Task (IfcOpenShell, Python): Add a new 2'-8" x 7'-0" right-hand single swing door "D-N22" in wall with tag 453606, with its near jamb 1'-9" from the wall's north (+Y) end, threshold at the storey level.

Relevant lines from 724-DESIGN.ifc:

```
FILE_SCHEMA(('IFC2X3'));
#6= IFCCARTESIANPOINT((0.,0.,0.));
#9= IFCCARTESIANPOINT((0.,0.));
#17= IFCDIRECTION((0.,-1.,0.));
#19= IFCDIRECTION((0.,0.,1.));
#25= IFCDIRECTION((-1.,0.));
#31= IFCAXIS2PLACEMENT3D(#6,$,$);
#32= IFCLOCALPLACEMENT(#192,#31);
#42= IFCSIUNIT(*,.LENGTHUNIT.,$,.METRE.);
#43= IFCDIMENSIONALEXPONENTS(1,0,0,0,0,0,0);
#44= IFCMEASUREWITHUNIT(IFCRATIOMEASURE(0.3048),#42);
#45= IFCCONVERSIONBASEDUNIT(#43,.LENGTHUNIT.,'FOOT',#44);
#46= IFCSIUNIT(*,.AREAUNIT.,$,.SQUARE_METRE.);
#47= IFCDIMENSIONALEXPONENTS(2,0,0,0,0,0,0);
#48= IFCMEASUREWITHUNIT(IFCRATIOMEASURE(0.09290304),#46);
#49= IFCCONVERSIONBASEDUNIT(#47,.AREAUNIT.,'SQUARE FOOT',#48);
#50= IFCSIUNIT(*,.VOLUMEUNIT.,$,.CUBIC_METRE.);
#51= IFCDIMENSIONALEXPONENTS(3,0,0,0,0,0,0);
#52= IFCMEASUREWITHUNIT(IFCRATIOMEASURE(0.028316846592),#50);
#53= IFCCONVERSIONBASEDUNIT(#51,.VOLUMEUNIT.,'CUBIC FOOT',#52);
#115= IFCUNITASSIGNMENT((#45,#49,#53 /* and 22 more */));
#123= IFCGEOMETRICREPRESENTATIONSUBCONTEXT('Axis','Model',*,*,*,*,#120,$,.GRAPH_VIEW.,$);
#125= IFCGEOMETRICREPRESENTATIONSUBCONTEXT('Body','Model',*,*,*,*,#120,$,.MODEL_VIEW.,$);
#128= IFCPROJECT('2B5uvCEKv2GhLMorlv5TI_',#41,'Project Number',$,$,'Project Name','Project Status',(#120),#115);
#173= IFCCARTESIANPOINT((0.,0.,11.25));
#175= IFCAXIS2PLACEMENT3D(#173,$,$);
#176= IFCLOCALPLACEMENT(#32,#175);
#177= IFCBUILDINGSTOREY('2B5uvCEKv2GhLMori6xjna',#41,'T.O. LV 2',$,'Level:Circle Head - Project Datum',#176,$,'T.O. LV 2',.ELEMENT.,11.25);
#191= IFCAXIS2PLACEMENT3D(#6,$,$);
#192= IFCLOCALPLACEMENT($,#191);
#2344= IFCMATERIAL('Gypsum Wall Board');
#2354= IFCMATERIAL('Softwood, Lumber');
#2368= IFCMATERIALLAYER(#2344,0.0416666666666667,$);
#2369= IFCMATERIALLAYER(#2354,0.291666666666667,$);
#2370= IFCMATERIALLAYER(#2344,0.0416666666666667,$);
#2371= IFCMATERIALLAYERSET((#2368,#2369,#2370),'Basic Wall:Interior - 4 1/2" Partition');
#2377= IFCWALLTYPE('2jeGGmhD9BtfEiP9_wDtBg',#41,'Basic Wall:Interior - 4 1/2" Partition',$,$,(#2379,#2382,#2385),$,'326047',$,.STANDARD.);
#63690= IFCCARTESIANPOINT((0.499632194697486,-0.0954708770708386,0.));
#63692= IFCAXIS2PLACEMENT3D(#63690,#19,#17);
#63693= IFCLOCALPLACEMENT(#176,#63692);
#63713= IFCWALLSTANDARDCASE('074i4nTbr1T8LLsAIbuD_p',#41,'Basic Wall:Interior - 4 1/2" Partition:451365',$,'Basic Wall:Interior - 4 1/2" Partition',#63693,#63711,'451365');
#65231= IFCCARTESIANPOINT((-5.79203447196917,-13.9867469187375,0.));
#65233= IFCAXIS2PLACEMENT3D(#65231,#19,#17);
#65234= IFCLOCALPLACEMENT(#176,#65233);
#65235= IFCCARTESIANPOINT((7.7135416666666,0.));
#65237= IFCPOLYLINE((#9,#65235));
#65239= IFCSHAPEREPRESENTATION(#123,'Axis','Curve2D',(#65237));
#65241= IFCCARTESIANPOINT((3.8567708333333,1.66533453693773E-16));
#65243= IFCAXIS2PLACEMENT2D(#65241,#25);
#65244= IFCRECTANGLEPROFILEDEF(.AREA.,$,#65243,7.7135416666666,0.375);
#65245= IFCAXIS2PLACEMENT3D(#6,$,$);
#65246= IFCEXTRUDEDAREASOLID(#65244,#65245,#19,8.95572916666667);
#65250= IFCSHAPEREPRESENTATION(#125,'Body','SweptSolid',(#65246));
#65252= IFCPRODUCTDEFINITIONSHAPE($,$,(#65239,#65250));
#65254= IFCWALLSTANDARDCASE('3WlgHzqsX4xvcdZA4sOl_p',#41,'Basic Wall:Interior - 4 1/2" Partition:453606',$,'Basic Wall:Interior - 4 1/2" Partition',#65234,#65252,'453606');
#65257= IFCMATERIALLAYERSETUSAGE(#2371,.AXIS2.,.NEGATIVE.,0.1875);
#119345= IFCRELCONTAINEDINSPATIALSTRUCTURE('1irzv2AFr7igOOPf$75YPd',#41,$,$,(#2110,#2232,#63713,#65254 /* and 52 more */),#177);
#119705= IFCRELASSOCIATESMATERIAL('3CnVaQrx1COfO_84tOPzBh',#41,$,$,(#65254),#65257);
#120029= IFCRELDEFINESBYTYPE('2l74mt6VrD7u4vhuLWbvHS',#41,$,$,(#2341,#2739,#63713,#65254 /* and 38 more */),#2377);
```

```python
import numpy as np
import ifcopenshell
import ifcopenshell.api.feature
import ifcopenshell.api.geometry
import ifcopenshell.api.root
import ifcopenshell.api.spatial
import ifcopenshell.api.type
import ifcopenshell.geom
import ifcopenshell.util.element
import ifcopenshell.util.placement
import ifcopenshell.util.representation
import ifcopenshell.util.shape
import ifcopenshell.util.unit

model = ifcopenshell.open("724-DESIGN.ifc")
unit_scale = ifcopenshell.util.unit.calculate_unit_scale(model)
settings = ifcopenshell.geom.settings()


def volume(element):
    """Net volume in cubic metres, openings subtracted."""
    shape = ifcopenshell.geom.create_shape(settings, element)
    return ifcopenshell.util.shape.get_volume(shape.geometry)


wall = model.by_id(65254)
storey = ifcopenshell.util.element.get_container(wall, ifc_class="IfcBuildingStorey")
context = ifcopenshell.util.representation.get_context(model, "Model", "Body", "MODEL_VIEW")
before = volume(wall)

width, height, from_end, sill = 0.8128, 2.1336, 0.5334, 0.0  # metres

# The wall runs along its own X axis, and the end named is its -X end.
wall_shape = ifcopenshell.geom.create_shape(settings, wall)
x, y, z = ifcopenshell.util.shape.get_vertices(wall_shape.geometry).T
start = x.min() + from_end
face, thickness = float(y.min()), float(y.max() - y.min())
wall_matrix = ifcopenshell.util.placement.get_local_placement(wall.ObjectPlacement)
level = ifcopenshell.util.placement.get_local_placement(storey.ObjectPlacement)[2, 3]


def in_wall(x, y):
    """Placement at x, y metres in the wall's axes, at sill height."""
    matrix = wall_matrix.copy()
    matrix[:, 3] = wall_matrix @ np.array([x / unit_scale, y / unit_scale, 0.0, 1.0])
    matrix[2, 3] = level + sill / unit_scale
    return matrix


# Opening: a box that overshoots both wall faces by 50 mm.
opening = ifcopenshell.api.root.create_entity(model, ifc_class="IfcOpeningElement")
box = ifcopenshell.api.geometry.add_wall_representation(
    model, context=context, length=width, height=height, thickness=thickness + 0.1
)
ifcopenshell.api.geometry.assign_representation(model, product=opening, representation=box)
ifcopenshell.api.geometry.edit_object_placement(model, product=opening, matrix=in_wall(start, face - 0.05), is_si=False)
ifcopenshell.api.feature.add_feature(model, feature=opening, element=wall)

door = ifcopenshell.api.root.create_entity(model, ifc_class="IfcDoor", name="D-N22")
door.OverallWidth, door.OverallHeight = width / unit_scale, height / unit_scale
body = ifcopenshell.api.geometry.add_door_representation(
    model,
    context=context,
    overall_width=door.OverallWidth,
    overall_height=door.OverallHeight,
    operation_type="SINGLE_SWING_RIGHT",
    lining_properties={"LiningDepth": thickness / unit_scale, "ThresholdDepth": thickness / unit_scale},
)
ifcopenshell.api.geometry.assign_representation(model, product=door, representation=body)
ifcopenshell.api.spatial.assign_container(model, products=[door], relating_structure=storey)
fills = ifcopenshell.api.feature.add_filling(model, opening=opening, element=door)
fills.OwnerHistory = door.OwnerHistory  # required in IFC2X3

# IFC2X3 keeps the operation on the door style.
style = ifcopenshell.api.root.create_entity(model, ifc_class="IfcDoorStyle", name="D-N22")
style.OperationType, style.ConstructionType = "SINGLE_SWING_RIGHT", "NOTDEFINED"
style.ParameterTakesPrecedence = style.Sizeable = False
ifcopenshell.api.type.assign_type(model, related_objects=[door], relating_type=style)

# The lining spans the wall, so the door starts at the wall face.
ifcopenshell.api.geometry.edit_object_placement(model, product=door, matrix=in_wall(start, face), is_si=False)

after = volume(wall)

print(f"wall volume {before:.3f} -> {after:.3f} m3")

model.write("724-DESIGN_rev.ifc")
```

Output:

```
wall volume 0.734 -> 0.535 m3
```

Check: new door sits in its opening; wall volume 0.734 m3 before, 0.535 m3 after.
